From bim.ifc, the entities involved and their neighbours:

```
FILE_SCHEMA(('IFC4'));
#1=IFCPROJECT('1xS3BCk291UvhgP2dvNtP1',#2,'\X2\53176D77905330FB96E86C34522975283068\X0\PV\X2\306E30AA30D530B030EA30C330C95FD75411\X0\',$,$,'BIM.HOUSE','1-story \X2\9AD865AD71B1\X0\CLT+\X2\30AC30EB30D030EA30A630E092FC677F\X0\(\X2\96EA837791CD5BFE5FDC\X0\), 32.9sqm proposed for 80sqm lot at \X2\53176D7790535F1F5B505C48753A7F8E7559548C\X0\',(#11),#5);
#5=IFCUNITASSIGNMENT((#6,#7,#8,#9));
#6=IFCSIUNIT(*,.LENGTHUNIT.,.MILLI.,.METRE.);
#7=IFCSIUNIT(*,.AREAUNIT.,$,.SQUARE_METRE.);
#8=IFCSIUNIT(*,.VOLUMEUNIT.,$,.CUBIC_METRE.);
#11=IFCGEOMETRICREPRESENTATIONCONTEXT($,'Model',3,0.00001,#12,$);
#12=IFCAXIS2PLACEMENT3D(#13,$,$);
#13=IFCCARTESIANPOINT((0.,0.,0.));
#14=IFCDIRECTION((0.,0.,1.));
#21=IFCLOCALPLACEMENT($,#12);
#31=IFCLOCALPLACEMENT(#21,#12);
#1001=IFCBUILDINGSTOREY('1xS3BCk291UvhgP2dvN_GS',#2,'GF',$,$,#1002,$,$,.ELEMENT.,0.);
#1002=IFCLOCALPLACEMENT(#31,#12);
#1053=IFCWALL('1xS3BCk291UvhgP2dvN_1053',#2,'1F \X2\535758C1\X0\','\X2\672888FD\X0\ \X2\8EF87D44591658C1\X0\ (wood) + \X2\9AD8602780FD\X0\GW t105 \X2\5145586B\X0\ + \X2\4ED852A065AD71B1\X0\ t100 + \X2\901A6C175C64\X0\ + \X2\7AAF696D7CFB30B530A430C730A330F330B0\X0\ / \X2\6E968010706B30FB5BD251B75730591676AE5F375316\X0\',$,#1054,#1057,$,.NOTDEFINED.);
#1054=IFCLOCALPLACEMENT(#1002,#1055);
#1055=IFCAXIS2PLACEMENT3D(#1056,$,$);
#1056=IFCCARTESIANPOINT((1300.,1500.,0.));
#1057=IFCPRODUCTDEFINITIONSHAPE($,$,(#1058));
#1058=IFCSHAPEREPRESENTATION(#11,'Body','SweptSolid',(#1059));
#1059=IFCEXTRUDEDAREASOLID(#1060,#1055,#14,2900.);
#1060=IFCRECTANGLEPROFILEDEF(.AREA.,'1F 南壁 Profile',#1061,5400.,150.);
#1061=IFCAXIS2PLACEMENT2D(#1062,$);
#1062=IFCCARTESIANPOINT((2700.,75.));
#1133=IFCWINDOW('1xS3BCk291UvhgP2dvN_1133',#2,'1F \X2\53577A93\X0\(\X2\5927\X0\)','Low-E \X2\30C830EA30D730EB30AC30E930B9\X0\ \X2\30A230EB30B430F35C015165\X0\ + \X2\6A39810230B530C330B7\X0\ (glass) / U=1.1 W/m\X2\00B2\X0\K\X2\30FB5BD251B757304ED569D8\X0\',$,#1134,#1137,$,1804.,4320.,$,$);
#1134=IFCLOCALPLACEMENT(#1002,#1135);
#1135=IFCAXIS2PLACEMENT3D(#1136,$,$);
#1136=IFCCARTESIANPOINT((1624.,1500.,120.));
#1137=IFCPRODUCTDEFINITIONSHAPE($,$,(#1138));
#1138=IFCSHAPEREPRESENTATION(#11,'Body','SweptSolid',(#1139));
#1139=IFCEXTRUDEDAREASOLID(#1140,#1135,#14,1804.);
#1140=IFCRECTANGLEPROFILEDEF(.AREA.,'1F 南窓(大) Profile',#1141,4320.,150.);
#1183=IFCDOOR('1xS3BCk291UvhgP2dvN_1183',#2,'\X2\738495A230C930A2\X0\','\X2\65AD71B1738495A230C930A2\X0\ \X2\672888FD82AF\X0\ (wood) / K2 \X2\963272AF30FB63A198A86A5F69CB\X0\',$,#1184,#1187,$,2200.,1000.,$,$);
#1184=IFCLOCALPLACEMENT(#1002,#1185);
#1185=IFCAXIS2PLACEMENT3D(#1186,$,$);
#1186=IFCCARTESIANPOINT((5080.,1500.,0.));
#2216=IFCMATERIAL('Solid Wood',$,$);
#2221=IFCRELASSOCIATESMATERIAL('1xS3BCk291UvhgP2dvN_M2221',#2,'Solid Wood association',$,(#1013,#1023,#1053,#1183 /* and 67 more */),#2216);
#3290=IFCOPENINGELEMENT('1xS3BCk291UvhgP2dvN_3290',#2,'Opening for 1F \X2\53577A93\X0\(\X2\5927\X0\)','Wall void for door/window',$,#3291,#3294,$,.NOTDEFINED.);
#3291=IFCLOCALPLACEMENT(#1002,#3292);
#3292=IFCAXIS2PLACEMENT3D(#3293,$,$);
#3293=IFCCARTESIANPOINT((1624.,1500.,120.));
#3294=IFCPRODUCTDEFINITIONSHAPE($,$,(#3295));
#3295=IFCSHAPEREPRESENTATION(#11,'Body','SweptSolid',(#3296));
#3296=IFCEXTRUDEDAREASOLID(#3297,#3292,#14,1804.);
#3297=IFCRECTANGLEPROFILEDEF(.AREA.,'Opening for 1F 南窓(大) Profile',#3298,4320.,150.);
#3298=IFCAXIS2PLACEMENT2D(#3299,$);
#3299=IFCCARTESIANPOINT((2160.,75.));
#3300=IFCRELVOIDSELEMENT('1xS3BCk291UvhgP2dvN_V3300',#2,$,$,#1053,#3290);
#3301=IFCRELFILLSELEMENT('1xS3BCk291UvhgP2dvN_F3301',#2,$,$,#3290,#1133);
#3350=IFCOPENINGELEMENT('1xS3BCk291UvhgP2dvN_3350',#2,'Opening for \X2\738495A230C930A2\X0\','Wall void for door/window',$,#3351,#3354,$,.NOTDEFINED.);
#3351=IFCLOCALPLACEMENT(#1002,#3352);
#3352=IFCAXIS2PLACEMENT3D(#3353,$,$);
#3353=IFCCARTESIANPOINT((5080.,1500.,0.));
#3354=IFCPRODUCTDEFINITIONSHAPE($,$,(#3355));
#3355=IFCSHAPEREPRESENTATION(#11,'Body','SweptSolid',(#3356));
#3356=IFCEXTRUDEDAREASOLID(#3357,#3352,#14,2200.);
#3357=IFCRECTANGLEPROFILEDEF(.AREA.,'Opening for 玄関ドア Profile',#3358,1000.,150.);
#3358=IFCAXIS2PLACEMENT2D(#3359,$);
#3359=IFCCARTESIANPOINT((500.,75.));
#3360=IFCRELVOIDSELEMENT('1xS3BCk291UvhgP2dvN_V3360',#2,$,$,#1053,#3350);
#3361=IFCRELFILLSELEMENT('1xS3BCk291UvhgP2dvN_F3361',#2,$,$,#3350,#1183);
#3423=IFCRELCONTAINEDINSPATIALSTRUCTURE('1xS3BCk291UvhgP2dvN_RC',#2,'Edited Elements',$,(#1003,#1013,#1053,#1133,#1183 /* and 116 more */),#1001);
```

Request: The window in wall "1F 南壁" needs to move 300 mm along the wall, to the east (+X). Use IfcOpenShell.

```python
import ifcopenshell
import ifcopenshell.api.geometry
import ifcopenshell.util.placement

model = ifcopenshell.open("bim.ifc")

window = model.by_guid("1xS3BCk291UvhgP2dvN_1133")
opening = window.FillsVoids[0].RelatingOpeningElement
wall = opening.VoidsElements[0].RelatingBuildingElement

wall_matrix = ifcopenshell.util.placement.get_local_placement(wall.ObjectPlacement)
shift = wall_matrix[:3, 0] * 300.0
before = ifcopenshell.util.placement.get_local_placement(window.ObjectPlacement)[:3, 3].copy()

# The window is not placed relative to its opening, so move both.
for product in (opening, window):
    matrix = ifcopenshell.util.placement.get_local_placement(product.ObjectPlacement)
    matrix[:3, 3] += shift
    ifcopenshell.api.geometry.edit_object_placement(model, product=product, matrix=matrix, is_si=False)

after = ifcopenshell.util.placement.get_local_placement(window.ObjectPlacement)[:3, 3]
print("window moved by", (after - before).round(3) + 0.0)

model.write("bim_updated.ifc")
```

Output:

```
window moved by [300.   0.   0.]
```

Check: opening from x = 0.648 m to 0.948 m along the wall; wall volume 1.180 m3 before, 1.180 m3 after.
